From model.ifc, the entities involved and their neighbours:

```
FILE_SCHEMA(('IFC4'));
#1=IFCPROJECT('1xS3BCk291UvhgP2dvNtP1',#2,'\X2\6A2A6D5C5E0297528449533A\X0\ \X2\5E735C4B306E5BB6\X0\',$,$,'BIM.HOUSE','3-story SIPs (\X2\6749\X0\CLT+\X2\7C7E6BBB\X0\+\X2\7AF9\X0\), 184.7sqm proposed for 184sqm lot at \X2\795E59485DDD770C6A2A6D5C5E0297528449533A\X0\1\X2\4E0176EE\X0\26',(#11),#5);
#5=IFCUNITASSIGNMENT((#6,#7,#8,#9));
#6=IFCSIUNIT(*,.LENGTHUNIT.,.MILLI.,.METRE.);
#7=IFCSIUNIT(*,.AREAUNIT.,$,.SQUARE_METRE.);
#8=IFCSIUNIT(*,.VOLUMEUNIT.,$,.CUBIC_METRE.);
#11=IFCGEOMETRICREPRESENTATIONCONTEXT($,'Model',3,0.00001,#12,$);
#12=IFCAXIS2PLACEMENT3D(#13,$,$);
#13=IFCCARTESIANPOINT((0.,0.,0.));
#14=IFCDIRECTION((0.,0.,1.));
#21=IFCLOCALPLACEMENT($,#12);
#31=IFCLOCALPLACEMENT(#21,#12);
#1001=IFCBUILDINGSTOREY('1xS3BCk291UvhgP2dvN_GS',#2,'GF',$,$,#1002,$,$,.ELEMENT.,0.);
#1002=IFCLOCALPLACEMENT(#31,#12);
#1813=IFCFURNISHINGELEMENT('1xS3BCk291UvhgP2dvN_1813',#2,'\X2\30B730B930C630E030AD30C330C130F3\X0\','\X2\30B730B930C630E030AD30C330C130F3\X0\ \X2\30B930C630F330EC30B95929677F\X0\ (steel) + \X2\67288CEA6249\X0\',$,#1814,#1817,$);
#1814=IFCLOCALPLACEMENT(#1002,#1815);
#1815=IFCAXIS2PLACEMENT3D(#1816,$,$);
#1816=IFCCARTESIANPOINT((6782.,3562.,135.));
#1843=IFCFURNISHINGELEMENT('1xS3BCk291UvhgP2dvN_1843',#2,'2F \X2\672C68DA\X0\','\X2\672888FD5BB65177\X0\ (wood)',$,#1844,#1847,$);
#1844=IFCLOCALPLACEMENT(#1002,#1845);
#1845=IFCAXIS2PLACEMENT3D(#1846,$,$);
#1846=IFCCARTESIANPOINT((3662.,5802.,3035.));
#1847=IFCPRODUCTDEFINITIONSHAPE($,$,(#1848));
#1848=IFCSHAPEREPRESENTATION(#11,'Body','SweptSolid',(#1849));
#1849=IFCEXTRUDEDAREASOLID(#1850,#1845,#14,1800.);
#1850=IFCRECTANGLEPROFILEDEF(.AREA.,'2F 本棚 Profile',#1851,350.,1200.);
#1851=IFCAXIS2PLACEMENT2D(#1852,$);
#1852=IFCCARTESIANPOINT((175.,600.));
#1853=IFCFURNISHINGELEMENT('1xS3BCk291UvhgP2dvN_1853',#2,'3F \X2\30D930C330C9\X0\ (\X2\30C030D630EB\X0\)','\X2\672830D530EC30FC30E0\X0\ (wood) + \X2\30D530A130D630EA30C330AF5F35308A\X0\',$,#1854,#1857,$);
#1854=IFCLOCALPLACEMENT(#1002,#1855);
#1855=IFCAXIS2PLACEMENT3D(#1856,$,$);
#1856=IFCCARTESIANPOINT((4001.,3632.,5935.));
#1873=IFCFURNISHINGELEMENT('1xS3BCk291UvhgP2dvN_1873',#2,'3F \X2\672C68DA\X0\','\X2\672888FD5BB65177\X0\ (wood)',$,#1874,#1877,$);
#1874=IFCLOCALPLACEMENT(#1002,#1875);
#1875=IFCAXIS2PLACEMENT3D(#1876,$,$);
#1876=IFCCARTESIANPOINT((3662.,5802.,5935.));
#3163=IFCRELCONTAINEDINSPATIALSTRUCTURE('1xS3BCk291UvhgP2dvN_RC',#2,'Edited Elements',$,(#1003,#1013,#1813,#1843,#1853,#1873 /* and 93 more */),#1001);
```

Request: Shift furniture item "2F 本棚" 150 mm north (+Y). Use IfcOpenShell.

```python
import ifcopenshell
import ifcopenshell.api.geometry
import ifcopenshell.util.placement
import ifcopenshell.util.unit

model = ifcopenshell.open("model.ifc")
unit_scale = ifcopenshell.util.unit.calculate_unit_scale(model)

item = model.by_id(1843)
matrix = ifcopenshell.util.placement.get_local_placement(item.ObjectPlacement)
matrix[1, 3] += 0.15 / unit_scale
ifcopenshell.api.geometry.edit_object_placement(model, product=item, matrix=matrix, is_si=False)

print(ifcopenshell.util.placement.get_local_placement(item.ObjectPlacement).round(3) + 0.0)

model.write("model_rev.ifc")
```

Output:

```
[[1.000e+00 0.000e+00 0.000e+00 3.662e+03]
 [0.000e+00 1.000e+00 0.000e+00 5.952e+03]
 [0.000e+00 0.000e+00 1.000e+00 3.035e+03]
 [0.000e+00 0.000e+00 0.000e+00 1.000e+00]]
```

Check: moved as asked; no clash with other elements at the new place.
